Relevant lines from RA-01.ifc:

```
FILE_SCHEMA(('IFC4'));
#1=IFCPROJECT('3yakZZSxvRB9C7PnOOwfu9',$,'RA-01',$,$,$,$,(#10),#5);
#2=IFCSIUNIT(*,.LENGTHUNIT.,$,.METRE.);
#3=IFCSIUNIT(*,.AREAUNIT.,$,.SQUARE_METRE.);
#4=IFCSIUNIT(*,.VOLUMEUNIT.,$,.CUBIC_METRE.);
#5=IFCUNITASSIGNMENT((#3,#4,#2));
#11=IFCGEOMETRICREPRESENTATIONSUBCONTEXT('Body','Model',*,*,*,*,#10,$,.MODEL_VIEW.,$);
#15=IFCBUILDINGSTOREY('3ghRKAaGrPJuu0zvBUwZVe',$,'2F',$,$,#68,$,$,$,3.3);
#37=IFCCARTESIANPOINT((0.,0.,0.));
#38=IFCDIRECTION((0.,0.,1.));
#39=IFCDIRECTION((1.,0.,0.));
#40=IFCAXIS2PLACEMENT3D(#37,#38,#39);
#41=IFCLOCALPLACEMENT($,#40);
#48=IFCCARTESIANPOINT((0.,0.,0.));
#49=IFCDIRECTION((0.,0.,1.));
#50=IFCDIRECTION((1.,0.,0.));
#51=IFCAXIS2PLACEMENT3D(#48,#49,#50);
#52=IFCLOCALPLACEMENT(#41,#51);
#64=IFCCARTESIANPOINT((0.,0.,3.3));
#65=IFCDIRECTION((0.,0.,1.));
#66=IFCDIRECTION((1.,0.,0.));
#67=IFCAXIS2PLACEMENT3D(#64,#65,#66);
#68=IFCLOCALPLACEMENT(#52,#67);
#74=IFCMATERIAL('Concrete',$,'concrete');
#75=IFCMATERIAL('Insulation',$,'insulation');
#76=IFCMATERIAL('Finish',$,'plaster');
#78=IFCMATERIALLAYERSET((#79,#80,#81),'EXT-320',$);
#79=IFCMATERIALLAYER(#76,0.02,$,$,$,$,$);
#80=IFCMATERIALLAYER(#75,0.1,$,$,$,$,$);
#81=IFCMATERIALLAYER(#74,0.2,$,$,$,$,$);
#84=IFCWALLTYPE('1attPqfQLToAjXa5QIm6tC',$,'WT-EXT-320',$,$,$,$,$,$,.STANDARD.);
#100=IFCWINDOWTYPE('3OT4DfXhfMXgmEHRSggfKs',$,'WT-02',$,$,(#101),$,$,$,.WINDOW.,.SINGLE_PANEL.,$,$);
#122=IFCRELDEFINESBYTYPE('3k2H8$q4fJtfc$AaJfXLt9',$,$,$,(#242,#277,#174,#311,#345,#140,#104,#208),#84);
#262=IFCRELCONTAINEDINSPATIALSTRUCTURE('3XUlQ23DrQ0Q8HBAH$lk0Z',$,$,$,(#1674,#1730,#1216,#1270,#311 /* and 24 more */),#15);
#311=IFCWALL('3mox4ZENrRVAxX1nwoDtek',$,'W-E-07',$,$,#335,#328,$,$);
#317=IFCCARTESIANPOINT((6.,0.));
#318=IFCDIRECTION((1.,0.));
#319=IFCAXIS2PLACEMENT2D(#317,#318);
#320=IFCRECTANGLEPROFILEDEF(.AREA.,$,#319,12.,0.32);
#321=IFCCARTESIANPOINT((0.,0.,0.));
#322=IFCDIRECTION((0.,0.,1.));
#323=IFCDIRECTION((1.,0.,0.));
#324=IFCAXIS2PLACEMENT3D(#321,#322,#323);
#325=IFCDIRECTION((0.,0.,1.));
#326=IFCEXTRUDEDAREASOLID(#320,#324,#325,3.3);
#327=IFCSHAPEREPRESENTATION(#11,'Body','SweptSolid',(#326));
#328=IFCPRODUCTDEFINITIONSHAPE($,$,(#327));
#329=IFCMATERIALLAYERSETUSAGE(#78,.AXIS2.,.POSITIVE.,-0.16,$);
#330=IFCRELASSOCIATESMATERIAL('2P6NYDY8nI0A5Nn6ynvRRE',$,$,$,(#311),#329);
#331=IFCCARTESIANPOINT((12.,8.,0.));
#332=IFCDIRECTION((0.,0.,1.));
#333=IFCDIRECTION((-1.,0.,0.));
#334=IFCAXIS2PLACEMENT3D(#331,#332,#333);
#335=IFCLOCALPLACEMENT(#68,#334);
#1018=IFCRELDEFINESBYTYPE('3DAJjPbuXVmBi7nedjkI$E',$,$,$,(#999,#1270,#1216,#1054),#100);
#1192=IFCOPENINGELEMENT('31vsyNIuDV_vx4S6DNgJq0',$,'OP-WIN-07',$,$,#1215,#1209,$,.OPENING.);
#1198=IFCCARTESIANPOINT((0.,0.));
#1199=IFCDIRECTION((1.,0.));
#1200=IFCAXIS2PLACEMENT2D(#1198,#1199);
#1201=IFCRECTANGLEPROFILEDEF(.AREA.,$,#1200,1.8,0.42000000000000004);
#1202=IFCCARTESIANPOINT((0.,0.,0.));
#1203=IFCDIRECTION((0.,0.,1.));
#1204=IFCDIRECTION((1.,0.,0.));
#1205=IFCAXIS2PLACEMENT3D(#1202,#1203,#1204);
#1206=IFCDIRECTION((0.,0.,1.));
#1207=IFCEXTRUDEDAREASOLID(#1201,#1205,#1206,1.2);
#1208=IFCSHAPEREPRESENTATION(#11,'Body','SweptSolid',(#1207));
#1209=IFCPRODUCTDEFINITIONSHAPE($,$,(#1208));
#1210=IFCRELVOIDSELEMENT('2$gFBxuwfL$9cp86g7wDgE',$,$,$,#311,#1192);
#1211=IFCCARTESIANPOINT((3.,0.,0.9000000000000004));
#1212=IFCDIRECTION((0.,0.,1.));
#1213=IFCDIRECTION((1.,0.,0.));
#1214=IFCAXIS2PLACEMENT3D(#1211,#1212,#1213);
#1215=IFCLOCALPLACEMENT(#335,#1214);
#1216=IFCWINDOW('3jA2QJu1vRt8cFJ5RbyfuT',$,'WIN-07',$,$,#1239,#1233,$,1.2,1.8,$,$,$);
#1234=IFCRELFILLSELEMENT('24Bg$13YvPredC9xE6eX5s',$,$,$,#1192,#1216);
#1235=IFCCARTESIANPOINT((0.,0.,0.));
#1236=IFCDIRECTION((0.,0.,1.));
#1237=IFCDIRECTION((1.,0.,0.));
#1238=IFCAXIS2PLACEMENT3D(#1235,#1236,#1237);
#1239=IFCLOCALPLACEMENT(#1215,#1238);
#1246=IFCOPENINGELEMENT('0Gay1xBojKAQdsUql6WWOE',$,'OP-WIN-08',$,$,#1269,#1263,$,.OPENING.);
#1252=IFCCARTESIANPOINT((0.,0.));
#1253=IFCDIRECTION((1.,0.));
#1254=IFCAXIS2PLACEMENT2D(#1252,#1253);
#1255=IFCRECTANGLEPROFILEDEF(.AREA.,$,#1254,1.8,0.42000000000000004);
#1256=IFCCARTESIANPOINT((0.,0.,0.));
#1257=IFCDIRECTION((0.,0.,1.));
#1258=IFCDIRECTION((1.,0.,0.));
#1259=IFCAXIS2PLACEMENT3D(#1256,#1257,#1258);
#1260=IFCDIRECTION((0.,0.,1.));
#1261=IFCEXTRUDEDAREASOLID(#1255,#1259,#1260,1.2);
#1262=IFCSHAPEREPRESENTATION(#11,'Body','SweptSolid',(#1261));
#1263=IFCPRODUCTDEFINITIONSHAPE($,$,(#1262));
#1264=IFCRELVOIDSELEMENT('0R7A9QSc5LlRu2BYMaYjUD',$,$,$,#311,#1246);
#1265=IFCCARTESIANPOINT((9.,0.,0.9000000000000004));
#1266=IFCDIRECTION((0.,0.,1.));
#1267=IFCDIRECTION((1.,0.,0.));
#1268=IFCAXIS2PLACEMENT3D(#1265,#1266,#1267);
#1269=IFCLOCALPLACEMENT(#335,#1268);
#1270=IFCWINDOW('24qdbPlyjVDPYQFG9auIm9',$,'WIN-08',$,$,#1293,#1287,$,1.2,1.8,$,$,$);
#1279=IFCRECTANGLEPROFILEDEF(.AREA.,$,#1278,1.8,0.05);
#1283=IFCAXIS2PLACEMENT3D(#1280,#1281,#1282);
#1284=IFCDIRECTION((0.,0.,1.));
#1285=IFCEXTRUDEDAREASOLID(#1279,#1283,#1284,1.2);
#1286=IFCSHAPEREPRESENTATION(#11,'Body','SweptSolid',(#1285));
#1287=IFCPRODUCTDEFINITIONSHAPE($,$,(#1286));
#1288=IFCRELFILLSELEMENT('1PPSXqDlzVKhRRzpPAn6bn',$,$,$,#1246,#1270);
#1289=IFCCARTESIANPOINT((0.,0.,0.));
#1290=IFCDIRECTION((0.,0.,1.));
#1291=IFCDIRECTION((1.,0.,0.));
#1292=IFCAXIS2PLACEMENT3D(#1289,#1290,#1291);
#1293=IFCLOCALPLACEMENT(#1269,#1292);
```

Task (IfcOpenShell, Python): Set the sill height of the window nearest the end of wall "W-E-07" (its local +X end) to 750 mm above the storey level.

```python
import numpy as np
import ifcopenshell
import ifcopenshell.api.geometry
import ifcopenshell.geom
import ifcopenshell.util.element
import ifcopenshell.util.placement
import ifcopenshell.util.shape
import ifcopenshell.util.unit

model = ifcopenshell.open("RA-01.ifc")
unit_scale = ifcopenshell.util.unit.calculate_unit_scale(model)

window = model.by_id(1270)
opening = window.FillsVoids[0].RelatingOpeningElement
storey = ifcopenshell.util.element.get_container(window, ifc_class="IfcBuildingStorey")
level = ifcopenshell.util.placement.get_local_placement(storey.ObjectPlacement)[2, 3]

# The opening's origin need not be at the sill, so measure its lowest point.
shape = ifcopenshell.geom.create_shape(ifcopenshell.geom.settings(), opening)
bottom = ifcopenshell.util.shape.get_shape_bottom_elevation(shape, shape.geometry) / unit_scale
dz = level + 0.75 / unit_scale - bottom

shift = np.array([0.0, 0.0, dz])
# The window is placed relative to its opening, so it follows when the opening moves.
matrix = ifcopenshell.util.placement.get_local_placement(opening.ObjectPlacement)
matrix[:3, 3] += shift
ifcopenshell.api.geometry.edit_object_placement(
    model, product=opening, matrix=matrix, is_si=False, should_transform_children=True
)

print(f"moved by {dz * unit_scale:+.3f} m")

model.write("RA-01-out.ifc")
```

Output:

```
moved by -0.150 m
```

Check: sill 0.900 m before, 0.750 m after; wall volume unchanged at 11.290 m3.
